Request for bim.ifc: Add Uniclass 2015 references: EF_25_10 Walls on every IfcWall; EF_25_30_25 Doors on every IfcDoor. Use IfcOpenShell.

First a look at what the model holds.

```python
import ifcopenshell

model = ifcopenshell.open("bim.ifc")
print(model.schema)
print("classifications:", [c.Name for c in model.by_type("IfcClassification")])
for ifc_class in ("IfcDoor", "IfcRoof", "IfcStair", "IfcWall", "IfcWindow"):
    print(ifc_class, len(model.by_type(ifc_class)))
```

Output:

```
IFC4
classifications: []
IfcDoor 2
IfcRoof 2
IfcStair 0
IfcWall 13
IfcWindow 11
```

```python
import ifcopenshell
import ifcopenshell.api.classification

model = ifcopenshell.open("bim.ifc")

system = ifcopenshell.api.classification.add_classification(model, classification="Uniclass 2015")

codes = {
    "IfcWall": ("EF_25_10", "Walls"),
    "IfcDoor": ("EF_25_30_25", "Doors"),
}
for ifc_class, (code, name) in codes.items():
    products = model.by_type(ifc_class)
    ifcopenshell.api.classification.add_reference(
        model, products=products, classification=system, identification=code, name=name
    )
    print(code, len(products))

model.write("bim_rev.ifc")
```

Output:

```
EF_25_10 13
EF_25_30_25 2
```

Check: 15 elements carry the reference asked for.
